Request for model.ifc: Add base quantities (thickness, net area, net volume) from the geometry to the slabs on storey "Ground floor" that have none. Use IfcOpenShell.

First a look at what the model holds.

```python
import ifcopenshell
import ifcopenshell.util.element
import ifcopenshell.util.unit

model = ifcopenshell.open("model.ifc")
print(model.schema)
for unit_type in ("LENGTHUNIT", "AREAUNIT", "VOLUMEUNIT"):
    print(unit_type, ifcopenshell.util.unit.calculate_unit_scale(model, unit_type))
storey = next(s for s in model.by_type("IfcBuildingStorey") if s.Name == "Ground floor")
slabs = [e for e in ifcopenshell.util.element.get_decomposition(storey) if e.is_a("IfcSlab")]
for e in sorted(slabs, key=lambda e: e.id()):
    print(e.id(), e.is_a(), e.Name, list(ifcopenshell.util.element.get_psets(e, qtos_only=True)), sep=" | ")
```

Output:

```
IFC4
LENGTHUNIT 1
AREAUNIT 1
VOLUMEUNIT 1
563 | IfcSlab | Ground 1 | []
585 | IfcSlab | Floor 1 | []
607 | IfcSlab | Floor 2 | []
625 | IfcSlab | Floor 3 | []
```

```python
import ifcopenshell
import ifcopenshell.api.pset
import ifcopenshell.geom
import ifcopenshell.util.element
import ifcopenshell.util.shape
import ifcopenshell.util.unit

model = ifcopenshell.open("model.ifc")
unit_scale = ifcopenshell.util.unit.calculate_unit_scale(model)
area_scale = ifcopenshell.util.unit.calculate_unit_scale(model, "AREAUNIT")
volume_scale = ifcopenshell.util.unit.calculate_unit_scale(model, "VOLUMEUNIT")
settings = ifcopenshell.geom.settings()

storey = next(s for s in model.by_type("IfcBuildingStorey") if s.Name == "Ground floor")
slabs = [e for e in ifcopenshell.util.element.get_decomposition(storey) if e.is_a("IfcSlab")]

for e in sorted(slabs, key=lambda e: e.id()):
    if ifcopenshell.util.element.get_psets(e, qtos_only=True, should_inherit=False):
        continue
    # Geometry comes back in metres, in the element's own axes.
    shape = ifcopenshell.geom.create_shape(settings, e)
    values = {
        "Width": ifcopenshell.util.shape.get_z(shape.geometry) / unit_scale,
        "NetArea": ifcopenshell.util.shape.get_footprint_area(shape.geometry) / area_scale,
        "NetVolume": ifcopenshell.util.shape.get_volume(shape.geometry) / volume_scale,
    }
    qto = ifcopenshell.api.pset.add_qto(model, product=e, name="Qto_SlabBaseQuantities")
    ifcopenshell.api.pset.edit_qto(model, qto=qto, properties=values)
    print(e.id(), {k: round(v, 3) for k, v in values.items()})

model.write("model_v2.ifc")
```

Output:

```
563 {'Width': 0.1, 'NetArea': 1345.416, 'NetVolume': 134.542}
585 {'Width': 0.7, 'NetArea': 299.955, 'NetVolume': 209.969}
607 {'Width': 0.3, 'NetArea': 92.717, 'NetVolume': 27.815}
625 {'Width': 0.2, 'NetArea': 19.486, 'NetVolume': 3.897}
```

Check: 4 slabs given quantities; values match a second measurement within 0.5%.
